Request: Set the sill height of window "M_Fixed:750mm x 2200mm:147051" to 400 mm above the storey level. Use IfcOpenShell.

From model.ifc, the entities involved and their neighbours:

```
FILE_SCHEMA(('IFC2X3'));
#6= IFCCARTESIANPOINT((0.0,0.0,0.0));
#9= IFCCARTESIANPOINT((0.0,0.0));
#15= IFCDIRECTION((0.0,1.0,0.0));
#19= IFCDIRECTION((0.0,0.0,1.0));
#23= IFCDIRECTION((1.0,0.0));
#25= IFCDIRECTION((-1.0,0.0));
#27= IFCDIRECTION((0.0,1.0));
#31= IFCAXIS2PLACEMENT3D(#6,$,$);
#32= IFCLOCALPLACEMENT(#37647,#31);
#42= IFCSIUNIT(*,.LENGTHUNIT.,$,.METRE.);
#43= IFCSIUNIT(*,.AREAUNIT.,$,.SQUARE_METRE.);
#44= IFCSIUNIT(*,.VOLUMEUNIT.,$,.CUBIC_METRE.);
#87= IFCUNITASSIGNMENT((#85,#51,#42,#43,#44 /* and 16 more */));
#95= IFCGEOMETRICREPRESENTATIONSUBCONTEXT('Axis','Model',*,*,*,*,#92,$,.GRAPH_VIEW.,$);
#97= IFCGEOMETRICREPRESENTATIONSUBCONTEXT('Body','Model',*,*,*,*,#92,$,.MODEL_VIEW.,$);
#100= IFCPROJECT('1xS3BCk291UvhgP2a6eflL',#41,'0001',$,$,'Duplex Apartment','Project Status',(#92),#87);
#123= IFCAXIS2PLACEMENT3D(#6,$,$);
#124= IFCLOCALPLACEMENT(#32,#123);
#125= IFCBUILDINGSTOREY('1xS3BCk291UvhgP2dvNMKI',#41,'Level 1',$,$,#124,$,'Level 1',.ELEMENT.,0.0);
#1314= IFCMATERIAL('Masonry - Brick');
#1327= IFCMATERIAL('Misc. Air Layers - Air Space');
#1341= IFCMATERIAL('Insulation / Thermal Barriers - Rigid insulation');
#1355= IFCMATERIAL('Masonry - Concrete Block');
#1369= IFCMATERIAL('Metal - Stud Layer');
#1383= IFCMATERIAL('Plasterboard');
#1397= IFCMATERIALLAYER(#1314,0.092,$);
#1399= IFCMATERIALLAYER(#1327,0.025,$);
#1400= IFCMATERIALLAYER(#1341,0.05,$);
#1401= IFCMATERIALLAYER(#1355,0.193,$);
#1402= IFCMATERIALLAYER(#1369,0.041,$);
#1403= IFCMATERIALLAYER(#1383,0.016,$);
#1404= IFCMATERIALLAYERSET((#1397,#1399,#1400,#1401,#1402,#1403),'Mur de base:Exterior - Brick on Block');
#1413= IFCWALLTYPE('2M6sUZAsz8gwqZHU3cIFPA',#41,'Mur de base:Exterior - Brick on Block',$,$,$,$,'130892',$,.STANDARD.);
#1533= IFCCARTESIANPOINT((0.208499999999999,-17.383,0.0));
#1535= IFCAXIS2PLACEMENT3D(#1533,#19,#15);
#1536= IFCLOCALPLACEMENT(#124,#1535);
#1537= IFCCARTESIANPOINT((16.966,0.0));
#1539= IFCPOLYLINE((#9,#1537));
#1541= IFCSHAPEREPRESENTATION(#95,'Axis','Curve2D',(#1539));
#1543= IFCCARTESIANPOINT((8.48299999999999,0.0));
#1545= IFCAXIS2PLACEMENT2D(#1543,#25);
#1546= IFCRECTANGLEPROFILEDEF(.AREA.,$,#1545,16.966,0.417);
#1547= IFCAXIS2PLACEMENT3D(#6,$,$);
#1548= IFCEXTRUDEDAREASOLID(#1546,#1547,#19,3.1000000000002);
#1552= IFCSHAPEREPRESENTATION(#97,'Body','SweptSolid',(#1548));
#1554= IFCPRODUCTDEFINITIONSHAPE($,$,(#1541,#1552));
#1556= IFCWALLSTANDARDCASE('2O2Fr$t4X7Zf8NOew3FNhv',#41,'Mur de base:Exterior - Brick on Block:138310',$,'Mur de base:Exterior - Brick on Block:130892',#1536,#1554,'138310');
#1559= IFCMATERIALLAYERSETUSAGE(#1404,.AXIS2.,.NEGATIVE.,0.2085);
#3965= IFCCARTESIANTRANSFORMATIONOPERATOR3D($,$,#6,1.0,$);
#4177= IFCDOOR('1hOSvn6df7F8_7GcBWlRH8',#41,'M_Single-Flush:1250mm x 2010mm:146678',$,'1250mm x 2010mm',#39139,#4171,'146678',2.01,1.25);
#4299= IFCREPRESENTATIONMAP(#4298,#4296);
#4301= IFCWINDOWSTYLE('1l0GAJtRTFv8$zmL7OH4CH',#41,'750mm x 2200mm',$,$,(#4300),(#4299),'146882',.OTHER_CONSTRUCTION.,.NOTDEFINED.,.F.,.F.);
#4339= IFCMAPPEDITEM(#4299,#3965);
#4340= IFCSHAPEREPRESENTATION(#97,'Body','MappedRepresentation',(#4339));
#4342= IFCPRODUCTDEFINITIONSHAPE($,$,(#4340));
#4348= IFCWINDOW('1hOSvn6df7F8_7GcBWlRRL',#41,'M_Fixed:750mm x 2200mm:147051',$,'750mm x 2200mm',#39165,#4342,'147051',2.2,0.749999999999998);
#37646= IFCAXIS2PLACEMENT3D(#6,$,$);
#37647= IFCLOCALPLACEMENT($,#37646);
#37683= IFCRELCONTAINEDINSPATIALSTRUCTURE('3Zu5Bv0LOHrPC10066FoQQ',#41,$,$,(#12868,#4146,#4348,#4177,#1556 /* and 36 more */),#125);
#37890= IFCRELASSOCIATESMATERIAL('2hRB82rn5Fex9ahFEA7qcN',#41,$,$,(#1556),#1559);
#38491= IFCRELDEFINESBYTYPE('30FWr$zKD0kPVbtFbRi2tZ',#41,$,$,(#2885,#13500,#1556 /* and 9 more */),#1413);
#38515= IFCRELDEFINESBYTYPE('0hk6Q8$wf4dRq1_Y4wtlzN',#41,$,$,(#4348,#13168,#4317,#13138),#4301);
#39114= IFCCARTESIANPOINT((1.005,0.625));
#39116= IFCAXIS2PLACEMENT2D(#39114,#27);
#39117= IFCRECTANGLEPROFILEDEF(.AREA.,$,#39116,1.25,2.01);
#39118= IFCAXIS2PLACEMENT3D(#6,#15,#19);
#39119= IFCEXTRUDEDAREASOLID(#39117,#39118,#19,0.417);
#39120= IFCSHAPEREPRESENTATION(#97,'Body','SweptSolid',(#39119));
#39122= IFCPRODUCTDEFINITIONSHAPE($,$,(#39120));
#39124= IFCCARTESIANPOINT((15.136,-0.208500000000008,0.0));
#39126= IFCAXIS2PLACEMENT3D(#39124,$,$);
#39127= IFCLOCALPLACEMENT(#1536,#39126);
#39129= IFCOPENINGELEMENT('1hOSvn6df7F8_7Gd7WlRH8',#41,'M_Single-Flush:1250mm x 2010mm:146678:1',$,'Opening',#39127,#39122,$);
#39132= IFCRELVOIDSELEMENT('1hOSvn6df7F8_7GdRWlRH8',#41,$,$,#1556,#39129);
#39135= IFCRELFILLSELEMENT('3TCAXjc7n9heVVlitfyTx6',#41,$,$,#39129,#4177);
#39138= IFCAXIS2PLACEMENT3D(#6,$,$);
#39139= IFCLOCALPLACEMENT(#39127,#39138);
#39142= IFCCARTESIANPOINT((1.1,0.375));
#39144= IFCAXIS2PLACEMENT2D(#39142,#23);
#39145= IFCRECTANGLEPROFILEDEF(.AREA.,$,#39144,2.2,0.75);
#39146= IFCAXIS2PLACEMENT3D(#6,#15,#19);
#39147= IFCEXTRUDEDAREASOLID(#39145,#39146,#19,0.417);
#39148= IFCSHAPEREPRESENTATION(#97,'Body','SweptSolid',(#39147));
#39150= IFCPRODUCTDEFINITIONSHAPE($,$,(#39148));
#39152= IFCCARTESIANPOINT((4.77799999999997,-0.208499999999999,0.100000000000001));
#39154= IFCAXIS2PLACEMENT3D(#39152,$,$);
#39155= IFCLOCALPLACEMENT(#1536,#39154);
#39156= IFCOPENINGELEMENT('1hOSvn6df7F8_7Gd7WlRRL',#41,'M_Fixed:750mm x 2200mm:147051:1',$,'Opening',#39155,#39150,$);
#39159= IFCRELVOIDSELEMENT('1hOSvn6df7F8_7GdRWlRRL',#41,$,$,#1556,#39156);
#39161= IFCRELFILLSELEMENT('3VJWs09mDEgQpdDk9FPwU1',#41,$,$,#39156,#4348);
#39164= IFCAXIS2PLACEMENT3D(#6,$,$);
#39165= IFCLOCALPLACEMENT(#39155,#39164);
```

```python
import numpy as np
import ifcopenshell
import ifcopenshell.api.geometry
import ifcopenshell.geom
import ifcopenshell.util.element
import ifcopenshell.util.placement
import ifcopenshell.util.shape
import ifcopenshell.util.unit

model = ifcopenshell.open("model.ifc")
unit_scale = ifcopenshell.util.unit.calculate_unit_scale(model)

window = model.by_id(4348)
opening = window.FillsVoids[0].RelatingOpeningElement
storey = ifcopenshell.util.element.get_container(window, ifc_class="IfcBuildingStorey")
level = ifcopenshell.util.placement.get_local_placement(storey.ObjectPlacement)[2, 3]

# The opening's origin need not be at the sill, so measure its lowest point.
shape = ifcopenshell.geom.create_shape(ifcopenshell.geom.settings(), opening)
bottom = ifcopenshell.util.shape.get_shape_bottom_elevation(shape, shape.geometry) / unit_scale
dz = level + 0.4 / unit_scale - bottom

shift = np.array([0.0, 0.0, dz])
# The window is placed relative to its opening, so it follows when the opening moves.
matrix = ifcopenshell.util.placement.get_local_placement(opening.ObjectPlacement)
matrix[:3, 3] += shift
ifcopenshell.api.geometry.edit_object_placement(
    model, product=opening, matrix=matrix, is_si=False, should_transform_children=True
)

print(f"moved by {dz * unit_scale:+.3f} m")

model.write("model_edited.ifc")
```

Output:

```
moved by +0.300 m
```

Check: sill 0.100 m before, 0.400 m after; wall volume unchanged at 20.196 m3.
